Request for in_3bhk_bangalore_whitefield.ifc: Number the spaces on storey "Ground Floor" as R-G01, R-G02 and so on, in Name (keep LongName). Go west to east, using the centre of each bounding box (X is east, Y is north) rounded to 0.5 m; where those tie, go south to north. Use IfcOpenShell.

First a look at what the model holds.

```python
import ifcopenshell
import ifcopenshell.util.element
import ifcopenshell.util.placement

model = ifcopenshell.open("in_3bhk_bangalore_whitefield.ifc")
print(model.schema)
storey = next(s for s in model.by_type("IfcBuildingStorey") if s.Name == "Ground Floor")
spaces = [e for e in ifcopenshell.util.element.get_decomposition(storey) if e.is_a("IfcSpace")]
for e in sorted(spaces, key=lambda e: e.id()):
    origin = ifcopenshell.util.placement.get_local_placement(e.ObjectPlacement)[:3, 3]
    print(e.id(), e.Name, e.LongName, origin.round(2) + 0.0, sep=" | ")
```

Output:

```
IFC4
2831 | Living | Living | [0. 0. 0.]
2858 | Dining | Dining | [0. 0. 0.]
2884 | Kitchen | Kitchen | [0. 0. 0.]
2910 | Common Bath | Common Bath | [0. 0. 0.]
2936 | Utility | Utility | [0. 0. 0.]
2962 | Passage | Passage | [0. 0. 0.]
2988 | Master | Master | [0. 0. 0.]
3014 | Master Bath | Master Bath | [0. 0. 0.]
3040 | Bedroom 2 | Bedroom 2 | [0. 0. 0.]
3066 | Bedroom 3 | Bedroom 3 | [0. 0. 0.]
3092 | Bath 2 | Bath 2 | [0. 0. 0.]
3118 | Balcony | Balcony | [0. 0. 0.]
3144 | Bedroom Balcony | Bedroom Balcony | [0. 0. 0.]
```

```python
import ifcopenshell
import ifcopenshell.geom
import ifcopenshell.util.element
import ifcopenshell.util.shape

model = ifcopenshell.open("in_3bhk_bangalore_whitefield.ifc")
settings = ifcopenshell.geom.settings()
settings.set("use-world-coords", True)


def centre(element):
    shape = ifcopenshell.geom.create_shape(settings, element)
    return ifcopenshell.util.shape.get_bbox_centroid(shape.geometry)


storey = next(s for s in model.by_type("IfcBuildingStorey") if s.Name == "Ground Floor")
spaces = [e for e in ifcopenshell.util.element.get_decomposition(storey) if e.is_a("IfcSpace")]

# Insertion points can sit at a corner or the storey origin, so sort by the geometry (in metres).
centres = {e: centre(e) for e in spaces}
spaces.sort(key=lambda e: (round(centres[e][0] / 0.5), centres[e][1]))

for i, e in enumerate(spaces, start=1):
    number = f"R-G{i:02d}"
    e.Name = number
    print(e.id(), number)

model.write("in_3bhk_bangalore_whitefield_edited.ifc")
```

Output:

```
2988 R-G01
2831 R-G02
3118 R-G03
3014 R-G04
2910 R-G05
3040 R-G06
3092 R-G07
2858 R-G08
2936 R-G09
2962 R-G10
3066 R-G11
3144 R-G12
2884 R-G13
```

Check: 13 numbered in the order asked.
